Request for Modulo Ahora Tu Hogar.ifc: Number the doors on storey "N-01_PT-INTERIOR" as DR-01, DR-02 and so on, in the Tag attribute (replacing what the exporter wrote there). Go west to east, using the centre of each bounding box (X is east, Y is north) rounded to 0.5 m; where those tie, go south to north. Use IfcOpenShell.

First a look at what the model holds.

```python
import ifcopenshell
import ifcopenshell.util.element
import ifcopenshell.util.placement

model = ifcopenshell.open("Modulo Ahora Tu Hogar.ifc")
print(model.schema)
storey = next(s for s in model.by_type("IfcBuildingStorey") if s.Name == "N-01_PT-INTERIOR")
doors = [e for e in ifcopenshell.util.element.get_decomposition(storey) if e.is_a("IfcDoor")]
for e in sorted(doors, key=lambda e: e.id()):
    origin = ifcopenshell.util.placement.get_local_placement(e.ObjectPlacement)[:3, 3]
    print(e.id(), e.Tag, e.Name, origin.round(2) + 0.0, sep=" | ")
```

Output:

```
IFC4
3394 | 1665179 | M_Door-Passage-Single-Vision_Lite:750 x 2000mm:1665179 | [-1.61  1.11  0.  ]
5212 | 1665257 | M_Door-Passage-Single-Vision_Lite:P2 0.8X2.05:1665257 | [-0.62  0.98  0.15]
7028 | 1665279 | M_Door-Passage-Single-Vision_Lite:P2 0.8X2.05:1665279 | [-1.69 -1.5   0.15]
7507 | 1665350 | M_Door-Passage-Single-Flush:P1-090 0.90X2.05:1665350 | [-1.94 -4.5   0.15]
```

```python
import ifcopenshell
import ifcopenshell.geom
import ifcopenshell.util.element
import ifcopenshell.util.shape

model = ifcopenshell.open("Modulo Ahora Tu Hogar.ifc")
settings = ifcopenshell.geom.settings()
settings.set("use-world-coords", True)


def centre(element):
    shape = ifcopenshell.geom.create_shape(settings, element)
    return ifcopenshell.util.shape.get_bbox_centroid(shape.geometry)


storey = next(s for s in model.by_type("IfcBuildingStorey") if s.Name == "N-01_PT-INTERIOR")
doors = [e for e in ifcopenshell.util.element.get_decomposition(storey) if e.is_a("IfcDoor")]

# Insertion points can sit at a corner or the storey origin, so sort by the geometry (in metres).
centres = {e: centre(e) for e in doors}
doors.sort(key=lambda e: (round(centres[e][0] / 0.5), centres[e][1]))

for i, e in enumerate(doors, start=1):
    number = f"DR-{i:02d}"
    e.Tag = number
    print(e.id(), number)

model.write("Modulo Ahora Tu Hogar_v2.ifc")
```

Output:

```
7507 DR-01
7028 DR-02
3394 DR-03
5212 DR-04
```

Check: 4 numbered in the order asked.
